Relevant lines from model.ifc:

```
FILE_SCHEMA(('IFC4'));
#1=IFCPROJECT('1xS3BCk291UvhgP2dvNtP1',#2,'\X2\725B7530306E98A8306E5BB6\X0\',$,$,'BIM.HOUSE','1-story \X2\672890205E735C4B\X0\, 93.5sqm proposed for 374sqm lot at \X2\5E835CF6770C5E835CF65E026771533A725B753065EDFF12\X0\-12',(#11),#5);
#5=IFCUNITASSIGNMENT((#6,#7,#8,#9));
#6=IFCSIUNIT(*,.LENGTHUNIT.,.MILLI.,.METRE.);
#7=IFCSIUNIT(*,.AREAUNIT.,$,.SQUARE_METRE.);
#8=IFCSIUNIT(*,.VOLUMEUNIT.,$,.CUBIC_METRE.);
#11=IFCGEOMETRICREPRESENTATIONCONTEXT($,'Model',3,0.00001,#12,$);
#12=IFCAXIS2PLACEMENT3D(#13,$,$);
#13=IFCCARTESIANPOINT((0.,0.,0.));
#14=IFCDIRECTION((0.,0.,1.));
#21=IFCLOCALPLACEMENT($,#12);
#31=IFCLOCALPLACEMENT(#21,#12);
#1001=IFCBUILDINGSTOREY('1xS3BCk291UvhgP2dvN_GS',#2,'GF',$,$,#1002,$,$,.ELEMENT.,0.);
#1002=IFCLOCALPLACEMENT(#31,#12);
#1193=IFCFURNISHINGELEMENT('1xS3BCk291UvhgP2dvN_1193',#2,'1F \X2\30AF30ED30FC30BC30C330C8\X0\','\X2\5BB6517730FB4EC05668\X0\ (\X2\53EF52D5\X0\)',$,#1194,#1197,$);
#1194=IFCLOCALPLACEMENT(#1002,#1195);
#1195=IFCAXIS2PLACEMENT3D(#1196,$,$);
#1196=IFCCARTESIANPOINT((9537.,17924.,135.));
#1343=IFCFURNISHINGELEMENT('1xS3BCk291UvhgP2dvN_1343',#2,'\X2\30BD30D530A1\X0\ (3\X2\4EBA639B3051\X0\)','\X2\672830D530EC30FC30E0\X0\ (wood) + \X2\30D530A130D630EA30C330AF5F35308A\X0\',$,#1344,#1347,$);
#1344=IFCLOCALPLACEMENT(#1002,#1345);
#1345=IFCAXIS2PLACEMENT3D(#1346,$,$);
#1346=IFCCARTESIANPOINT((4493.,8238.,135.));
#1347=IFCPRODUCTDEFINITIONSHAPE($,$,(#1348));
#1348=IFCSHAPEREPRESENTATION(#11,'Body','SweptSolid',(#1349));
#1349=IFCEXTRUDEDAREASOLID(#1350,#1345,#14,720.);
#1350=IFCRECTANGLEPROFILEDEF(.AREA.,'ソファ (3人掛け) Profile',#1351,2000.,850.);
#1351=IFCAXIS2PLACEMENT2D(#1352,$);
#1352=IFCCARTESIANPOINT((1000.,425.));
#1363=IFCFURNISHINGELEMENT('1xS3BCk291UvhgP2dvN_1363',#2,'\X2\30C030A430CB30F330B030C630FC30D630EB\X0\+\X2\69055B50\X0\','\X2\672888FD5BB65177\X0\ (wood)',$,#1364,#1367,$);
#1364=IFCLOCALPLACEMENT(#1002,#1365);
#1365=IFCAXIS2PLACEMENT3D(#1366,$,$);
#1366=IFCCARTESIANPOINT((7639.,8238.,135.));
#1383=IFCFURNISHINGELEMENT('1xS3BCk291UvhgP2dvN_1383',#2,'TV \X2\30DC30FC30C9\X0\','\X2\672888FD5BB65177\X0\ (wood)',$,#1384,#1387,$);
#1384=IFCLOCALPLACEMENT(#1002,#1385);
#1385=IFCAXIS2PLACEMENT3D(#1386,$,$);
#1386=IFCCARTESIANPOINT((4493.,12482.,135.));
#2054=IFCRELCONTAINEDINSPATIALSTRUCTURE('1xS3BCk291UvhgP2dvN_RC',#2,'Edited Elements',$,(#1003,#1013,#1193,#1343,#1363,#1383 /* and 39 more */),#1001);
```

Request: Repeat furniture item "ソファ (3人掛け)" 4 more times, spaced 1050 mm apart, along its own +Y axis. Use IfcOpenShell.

```python
import ifcopenshell
import ifcopenshell.api.geometry
import ifcopenshell.api.root
import ifcopenshell.util.element
import ifcopenshell.util.placement

model = ifcopenshell.open("model.ifc")


def reuse_history(source, copy):
    """copy_class also copies each property set's owner history, people and application; keep the originals."""
    for rel in copy.IsDefinedBy:
        if rel.is_a("IfcRelDefinesByProperties") and (history := rel.RelatingPropertyDefinition.OwnerHistory):
            rel.RelatingPropertyDefinition.OwnerHistory = source.OwnerHistory
            ifcopenshell.util.element.remove_deep2(model, history)


source = model.by_id(1343)
base = ifcopenshell.util.placement.get_local_placement(source.ObjectPlacement)
step = base[:3, 1] * 1050.0

for i in range(1, 5):
    copy = ifcopenshell.api.root.copy_class(model, product=source)
    copy.Representation = ifcopenshell.util.element.copy_deep(
        model, source.Representation, exclude=["IfcGeometricRepresentationContext", "IfcRepresentationMap"]
    )
    reuse_history(source, copy)
    matrix = base.copy()
    matrix[:3, 3] += i * step
    print("added at", matrix[:3, 3].round(3) + 0.0)
    ifcopenshell.api.geometry.edit_object_placement(model, product=copy, matrix=matrix, is_si=False)

model.write("model_updated.ifc")
```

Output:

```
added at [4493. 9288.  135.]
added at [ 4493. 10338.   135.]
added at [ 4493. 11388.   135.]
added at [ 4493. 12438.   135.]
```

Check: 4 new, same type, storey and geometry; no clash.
